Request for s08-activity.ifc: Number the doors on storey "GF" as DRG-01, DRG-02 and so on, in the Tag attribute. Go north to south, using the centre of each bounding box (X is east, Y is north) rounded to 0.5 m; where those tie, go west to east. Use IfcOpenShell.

First a look at what the model holds.

```python
import ifcopenshell
import ifcopenshell.util.element
import ifcopenshell.util.placement

model = ifcopenshell.open("s08-activity.ifc")
print(model.schema)
storey = next(s for s in model.by_type("IfcBuildingStorey") if s.Name == "GF")
doors = [e for e in ifcopenshell.util.element.get_decomposition(storey) if e.is_a("IfcDoor")]
for e in sorted(doors, key=lambda e: e.id()):
    origin = ifcopenshell.util.placement.get_local_placement(e.ObjectPlacement)[:3, 3]
    print(e.id(), e.Tag, e.Name, origin.round(2) + 0.0, sep=" | ")
```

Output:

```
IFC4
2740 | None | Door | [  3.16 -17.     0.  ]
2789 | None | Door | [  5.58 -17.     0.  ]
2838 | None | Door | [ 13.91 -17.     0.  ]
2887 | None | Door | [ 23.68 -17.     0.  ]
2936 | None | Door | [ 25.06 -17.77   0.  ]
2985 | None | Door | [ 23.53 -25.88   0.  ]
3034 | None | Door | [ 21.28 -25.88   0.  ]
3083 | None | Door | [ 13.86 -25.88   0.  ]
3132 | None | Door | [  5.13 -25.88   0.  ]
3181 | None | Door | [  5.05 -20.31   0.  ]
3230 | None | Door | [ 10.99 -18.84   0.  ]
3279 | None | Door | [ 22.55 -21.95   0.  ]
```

```python
import ifcopenshell
import ifcopenshell.geom
import ifcopenshell.util.element
import ifcopenshell.util.shape

model = ifcopenshell.open("s08-activity.ifc")
settings = ifcopenshell.geom.settings()
settings.set("use-world-coords", True)


def centre(element):
    shape = ifcopenshell.geom.create_shape(settings, element)
    return ifcopenshell.util.shape.get_bbox_centroid(shape.geometry)


storey = next(s for s in model.by_type("IfcBuildingStorey") if s.Name == "GF")
doors = [e for e in ifcopenshell.util.element.get_decomposition(storey) if e.is_a("IfcDoor")]

# Insertion points can sit at a corner or the storey origin, so sort by the geometry (in metres).
centres = {e: centre(e) for e in doors}
doors.sort(key=lambda e: (-round(centres[e][1] / 0.5), centres[e][0]))

for i, e in enumerate(doors, start=1):
    number = f"DRG-{i:02d}"
    e.Tag = number
    print(e.id(), number)

model.write("s08-activity-out.ifc")
```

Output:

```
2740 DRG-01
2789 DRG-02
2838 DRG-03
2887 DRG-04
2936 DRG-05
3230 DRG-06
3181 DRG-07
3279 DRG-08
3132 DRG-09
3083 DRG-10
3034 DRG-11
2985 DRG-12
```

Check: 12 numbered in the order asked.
